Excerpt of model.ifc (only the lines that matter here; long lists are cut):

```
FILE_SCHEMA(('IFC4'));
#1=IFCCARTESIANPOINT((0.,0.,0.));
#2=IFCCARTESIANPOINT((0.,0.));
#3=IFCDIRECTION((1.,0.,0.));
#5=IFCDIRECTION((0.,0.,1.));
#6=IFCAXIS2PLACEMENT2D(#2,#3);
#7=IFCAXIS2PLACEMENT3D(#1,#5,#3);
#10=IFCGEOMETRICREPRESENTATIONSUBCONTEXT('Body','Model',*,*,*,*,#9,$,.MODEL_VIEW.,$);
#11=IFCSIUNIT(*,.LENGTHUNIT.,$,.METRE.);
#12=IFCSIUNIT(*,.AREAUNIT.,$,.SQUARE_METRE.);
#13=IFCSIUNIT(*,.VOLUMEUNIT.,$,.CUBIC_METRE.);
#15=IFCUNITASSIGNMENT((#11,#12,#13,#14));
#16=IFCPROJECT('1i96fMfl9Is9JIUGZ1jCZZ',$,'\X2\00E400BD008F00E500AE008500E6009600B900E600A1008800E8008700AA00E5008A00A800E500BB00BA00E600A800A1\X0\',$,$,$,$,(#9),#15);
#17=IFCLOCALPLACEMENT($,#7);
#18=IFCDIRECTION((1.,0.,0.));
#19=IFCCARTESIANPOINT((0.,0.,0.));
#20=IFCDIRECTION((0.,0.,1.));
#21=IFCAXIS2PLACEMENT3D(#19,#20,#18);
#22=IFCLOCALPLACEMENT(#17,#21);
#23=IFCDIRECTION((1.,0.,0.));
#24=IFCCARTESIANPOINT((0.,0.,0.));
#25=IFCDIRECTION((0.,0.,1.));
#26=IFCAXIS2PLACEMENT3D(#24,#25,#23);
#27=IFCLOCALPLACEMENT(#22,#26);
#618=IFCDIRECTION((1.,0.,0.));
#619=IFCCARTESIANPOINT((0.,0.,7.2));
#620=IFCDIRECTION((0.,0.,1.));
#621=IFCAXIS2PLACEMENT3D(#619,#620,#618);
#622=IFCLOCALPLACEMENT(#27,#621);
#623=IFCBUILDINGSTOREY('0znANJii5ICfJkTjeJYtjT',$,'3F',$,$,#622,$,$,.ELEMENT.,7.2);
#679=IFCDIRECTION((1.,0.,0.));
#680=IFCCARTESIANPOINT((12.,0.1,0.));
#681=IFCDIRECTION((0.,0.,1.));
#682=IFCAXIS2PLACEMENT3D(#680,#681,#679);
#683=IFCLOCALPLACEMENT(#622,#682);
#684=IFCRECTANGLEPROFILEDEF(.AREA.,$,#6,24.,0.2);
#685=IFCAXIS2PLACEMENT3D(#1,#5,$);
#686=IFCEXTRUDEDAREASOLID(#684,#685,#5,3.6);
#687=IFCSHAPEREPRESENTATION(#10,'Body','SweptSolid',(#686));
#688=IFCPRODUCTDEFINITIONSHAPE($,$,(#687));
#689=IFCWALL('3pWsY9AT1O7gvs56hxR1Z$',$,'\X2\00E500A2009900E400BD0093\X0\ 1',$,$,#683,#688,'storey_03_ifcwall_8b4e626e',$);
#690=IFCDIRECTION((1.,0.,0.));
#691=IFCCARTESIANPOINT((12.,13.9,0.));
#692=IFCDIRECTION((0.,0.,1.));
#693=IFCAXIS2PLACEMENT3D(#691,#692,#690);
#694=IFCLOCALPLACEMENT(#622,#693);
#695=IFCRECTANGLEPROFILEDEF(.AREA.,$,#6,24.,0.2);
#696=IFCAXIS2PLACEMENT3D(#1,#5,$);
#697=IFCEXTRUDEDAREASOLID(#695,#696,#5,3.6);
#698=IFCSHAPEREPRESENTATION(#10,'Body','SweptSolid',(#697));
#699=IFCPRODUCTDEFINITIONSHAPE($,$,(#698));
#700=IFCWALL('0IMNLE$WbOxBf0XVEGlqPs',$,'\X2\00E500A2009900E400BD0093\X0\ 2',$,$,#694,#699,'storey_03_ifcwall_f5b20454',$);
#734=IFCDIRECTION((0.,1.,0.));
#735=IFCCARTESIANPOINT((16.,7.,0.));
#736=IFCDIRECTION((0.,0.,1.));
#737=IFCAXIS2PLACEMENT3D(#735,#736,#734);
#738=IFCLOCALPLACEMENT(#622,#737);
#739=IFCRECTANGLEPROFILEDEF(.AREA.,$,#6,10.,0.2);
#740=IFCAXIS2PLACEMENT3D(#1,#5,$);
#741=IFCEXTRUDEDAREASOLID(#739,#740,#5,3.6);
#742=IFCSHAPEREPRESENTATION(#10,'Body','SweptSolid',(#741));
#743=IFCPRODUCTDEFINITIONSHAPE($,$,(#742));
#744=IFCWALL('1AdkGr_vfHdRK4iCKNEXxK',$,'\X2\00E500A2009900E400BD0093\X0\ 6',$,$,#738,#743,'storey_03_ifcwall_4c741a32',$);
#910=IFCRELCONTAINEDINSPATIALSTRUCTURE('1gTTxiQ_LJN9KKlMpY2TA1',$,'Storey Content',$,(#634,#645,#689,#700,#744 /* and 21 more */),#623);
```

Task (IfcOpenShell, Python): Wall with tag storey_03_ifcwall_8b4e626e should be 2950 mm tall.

```python
import ifcopenshell
import ifcopenshell.geom
import ifcopenshell.util.representation
import ifcopenshell.util.shape
import ifcopenshell.util.unit

model = ifcopenshell.open("model.ifc")
unit_scale = ifcopenshell.util.unit.calculate_unit_scale(model)
settings = ifcopenshell.geom.settings()


def volume(element):
    """Net volume in cubic metres, openings subtracted."""
    shape = ifcopenshell.geom.create_shape(settings, element)
    return ifcopenshell.util.shape.get_volume(shape.geometry)


wall = model.by_id(689)
before = volume(wall)

body = ifcopenshell.util.representation.get_representation(wall, "Model", "Body")
solid = body.Items[0]
old_height = solid.Depth
solid.Depth = 2.95 / unit_scale
after = volume(wall)

print(f"height {old_height:g} -> {solid.Depth:g}, volume {before:.3f} -> {after:.3f} m3")

model.write("model_edited.ifc")
```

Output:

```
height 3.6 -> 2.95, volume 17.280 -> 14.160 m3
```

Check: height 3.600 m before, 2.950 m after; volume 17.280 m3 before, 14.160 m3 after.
